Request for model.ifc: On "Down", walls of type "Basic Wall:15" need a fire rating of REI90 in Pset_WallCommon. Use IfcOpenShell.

First a look at what the model holds.

```python
import ifcopenshell
import ifcopenshell.util.element

model = ifcopenshell.open("model.ifc")
print(model.schema)
storey = next(s for s in model.by_type("IfcBuildingStorey") if s.Name == "Down")
walls = [e for e in ifcopenshell.util.element.get_decomposition(storey) if e.is_a("IfcWall")]
seen = {}
for e in walls:
    element_type = ifcopenshell.util.element.get_type(e)
    key = (element_type.Name if element_type != e and element_type else None, ifcopenshell.util.element.get_pset(e, "Pset_WallCommon", "FireRating"))
    seen[key] = seen.get(key, 0) + 1
for (name, value), count in sorted(seen.items(), key=str):
    print(count, "x", name, "|", value)
```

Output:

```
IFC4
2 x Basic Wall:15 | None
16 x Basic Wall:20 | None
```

```python
import ifcopenshell
import ifcopenshell.api.pset
import ifcopenshell.util.element

model = ifcopenshell.open("model.ifc")

storey = next(s for s in model.by_type("IfcBuildingStorey") if s.Name == "Down")
walls = [e for e in ifcopenshell.util.element.get_decomposition(storey) if e.is_a("IfcWall")]

count = 0
for e in walls:
    element_type = ifcopenshell.util.element.get_type(e)
    if element_type in (None, e) or element_type.Name != "Basic Wall:15":
        continue
    # add_pset returns the element's existing set when there is one.
    pset = ifcopenshell.api.pset.add_pset(model, product=e, name="Pset_WallCommon")
    ifcopenshell.api.pset.edit_pset(model, pset=pset, properties={"FireRating": "REI90"})
    count += 1

print(count, "walls updated")

model.write("model_updated.ifc")
```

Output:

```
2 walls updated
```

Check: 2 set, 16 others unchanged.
